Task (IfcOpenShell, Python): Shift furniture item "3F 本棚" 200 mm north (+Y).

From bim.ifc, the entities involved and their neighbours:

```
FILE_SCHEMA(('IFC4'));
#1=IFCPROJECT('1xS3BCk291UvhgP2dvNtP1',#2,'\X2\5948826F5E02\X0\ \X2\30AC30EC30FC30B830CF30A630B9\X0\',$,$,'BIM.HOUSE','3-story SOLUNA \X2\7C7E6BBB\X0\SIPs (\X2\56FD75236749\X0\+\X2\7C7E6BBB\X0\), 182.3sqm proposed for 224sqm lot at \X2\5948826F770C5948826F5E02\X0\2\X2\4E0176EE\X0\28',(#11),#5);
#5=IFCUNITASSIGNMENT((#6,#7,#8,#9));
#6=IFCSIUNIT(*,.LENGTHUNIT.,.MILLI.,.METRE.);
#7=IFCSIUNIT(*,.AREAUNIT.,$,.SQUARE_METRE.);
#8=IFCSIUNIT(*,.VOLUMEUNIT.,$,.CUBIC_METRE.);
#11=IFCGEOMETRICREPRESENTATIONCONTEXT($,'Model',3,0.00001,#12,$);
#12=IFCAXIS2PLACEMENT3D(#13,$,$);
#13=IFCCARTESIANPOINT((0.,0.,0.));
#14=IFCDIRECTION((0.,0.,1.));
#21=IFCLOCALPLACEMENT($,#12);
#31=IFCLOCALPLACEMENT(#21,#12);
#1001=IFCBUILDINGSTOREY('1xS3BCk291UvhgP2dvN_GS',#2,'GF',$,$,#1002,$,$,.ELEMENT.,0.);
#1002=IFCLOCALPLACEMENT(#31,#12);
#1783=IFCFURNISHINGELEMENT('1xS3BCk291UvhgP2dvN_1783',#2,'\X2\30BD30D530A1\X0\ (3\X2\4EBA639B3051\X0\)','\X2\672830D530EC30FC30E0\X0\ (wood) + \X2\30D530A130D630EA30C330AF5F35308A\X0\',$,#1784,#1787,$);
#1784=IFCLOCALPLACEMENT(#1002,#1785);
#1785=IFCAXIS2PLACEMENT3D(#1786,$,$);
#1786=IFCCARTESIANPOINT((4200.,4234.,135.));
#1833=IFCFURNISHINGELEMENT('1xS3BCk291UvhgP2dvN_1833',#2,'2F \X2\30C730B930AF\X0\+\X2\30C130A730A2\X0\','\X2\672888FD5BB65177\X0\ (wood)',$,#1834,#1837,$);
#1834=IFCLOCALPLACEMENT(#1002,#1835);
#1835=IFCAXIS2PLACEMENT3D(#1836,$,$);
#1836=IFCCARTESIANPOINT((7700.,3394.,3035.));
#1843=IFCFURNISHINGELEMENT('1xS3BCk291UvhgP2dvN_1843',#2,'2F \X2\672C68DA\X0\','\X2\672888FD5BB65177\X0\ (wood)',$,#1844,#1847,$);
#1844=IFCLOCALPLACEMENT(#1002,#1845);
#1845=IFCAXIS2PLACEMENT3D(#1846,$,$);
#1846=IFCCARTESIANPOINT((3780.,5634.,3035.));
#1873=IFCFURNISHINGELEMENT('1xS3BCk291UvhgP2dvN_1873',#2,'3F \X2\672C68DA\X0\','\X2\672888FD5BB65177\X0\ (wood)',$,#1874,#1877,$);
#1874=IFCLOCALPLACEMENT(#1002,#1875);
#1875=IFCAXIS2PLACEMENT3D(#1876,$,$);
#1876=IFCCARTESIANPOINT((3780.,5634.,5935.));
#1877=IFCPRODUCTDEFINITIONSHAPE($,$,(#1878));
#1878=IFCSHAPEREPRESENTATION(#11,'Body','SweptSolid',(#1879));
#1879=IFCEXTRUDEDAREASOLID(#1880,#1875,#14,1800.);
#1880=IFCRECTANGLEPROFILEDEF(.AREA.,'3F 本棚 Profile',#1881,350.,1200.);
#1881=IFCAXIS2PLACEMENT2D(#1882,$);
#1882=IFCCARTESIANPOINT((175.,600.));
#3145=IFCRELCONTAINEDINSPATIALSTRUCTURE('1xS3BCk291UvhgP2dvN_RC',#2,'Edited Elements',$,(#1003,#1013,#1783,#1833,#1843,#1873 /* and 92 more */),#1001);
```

```python
import ifcopenshell
import ifcopenshell.api.geometry
import ifcopenshell.util.placement

model = ifcopenshell.open("bim.ifc")

item = model.by_id(1873)
matrix = ifcopenshell.util.placement.get_local_placement(item.ObjectPlacement)
matrix[1, 3] += 200.0
ifcopenshell.api.geometry.edit_object_placement(model, product=item, matrix=matrix, is_si=False)

print(ifcopenshell.util.placement.get_local_placement(item.ObjectPlacement).round(3) + 0.0)

model.write("bim_rev.ifc")
```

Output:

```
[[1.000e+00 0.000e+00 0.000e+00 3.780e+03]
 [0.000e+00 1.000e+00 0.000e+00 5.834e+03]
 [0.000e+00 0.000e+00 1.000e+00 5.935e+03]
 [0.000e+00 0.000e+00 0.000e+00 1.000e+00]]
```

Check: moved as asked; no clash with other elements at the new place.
